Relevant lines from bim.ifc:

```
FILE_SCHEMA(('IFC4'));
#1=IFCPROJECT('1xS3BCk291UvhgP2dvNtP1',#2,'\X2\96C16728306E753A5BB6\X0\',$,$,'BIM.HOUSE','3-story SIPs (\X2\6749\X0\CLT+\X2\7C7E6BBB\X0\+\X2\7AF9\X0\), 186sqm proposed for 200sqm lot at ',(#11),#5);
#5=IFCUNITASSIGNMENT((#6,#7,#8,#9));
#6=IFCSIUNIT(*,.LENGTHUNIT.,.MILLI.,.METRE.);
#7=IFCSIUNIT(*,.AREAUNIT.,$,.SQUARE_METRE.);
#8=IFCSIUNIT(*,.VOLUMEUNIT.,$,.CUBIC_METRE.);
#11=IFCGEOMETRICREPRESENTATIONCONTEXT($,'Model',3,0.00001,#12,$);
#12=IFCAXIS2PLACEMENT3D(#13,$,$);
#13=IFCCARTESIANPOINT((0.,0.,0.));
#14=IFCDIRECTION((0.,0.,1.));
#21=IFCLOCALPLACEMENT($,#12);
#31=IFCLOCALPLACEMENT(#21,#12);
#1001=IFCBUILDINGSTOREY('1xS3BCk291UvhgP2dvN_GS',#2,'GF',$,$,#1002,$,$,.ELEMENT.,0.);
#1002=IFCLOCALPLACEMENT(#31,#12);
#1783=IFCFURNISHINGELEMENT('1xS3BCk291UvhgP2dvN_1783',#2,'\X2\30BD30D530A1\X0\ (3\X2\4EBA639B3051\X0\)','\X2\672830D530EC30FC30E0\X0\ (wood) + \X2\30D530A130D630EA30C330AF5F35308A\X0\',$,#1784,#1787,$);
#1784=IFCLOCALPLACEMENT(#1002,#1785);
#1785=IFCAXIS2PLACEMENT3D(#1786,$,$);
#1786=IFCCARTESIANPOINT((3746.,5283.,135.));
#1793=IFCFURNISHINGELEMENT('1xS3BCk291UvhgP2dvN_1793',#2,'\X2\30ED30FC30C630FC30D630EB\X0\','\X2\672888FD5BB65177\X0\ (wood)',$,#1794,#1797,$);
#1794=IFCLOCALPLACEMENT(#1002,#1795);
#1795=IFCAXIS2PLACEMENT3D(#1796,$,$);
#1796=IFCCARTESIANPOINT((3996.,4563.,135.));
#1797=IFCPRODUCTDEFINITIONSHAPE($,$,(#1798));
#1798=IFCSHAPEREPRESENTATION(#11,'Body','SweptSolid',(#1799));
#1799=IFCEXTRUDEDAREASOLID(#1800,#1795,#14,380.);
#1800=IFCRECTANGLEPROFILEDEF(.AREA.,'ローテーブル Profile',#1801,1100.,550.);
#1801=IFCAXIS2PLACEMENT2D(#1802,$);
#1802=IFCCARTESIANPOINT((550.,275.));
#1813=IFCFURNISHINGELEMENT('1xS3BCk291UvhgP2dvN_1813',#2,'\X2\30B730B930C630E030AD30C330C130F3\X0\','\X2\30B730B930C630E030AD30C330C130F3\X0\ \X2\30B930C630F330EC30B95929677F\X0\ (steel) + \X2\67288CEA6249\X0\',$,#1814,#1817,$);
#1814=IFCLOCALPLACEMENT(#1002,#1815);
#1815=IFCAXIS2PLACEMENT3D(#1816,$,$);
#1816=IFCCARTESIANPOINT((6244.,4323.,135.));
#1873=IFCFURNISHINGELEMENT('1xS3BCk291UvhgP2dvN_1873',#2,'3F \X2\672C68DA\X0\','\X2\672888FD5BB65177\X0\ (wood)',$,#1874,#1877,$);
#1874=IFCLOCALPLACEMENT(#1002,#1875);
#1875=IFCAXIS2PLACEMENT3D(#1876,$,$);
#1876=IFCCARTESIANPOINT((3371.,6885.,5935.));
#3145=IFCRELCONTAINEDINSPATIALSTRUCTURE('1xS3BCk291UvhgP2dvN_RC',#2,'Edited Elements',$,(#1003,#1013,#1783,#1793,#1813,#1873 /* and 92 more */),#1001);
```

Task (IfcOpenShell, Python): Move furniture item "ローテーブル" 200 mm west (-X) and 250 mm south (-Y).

```python
import ifcopenshell
import ifcopenshell.api.geometry
import ifcopenshell.util.placement
import ifcopenshell.util.unit

model = ifcopenshell.open("bim.ifc")
unit_scale = ifcopenshell.util.unit.calculate_unit_scale(model)

item = model.by_guid("1xS3BCk291UvhgP2dvN_1793")
matrix = ifcopenshell.util.placement.get_local_placement(item.ObjectPlacement)
matrix[0, 3] -= 0.2 / unit_scale
matrix[1, 3] -= 0.25 / unit_scale
ifcopenshell.api.geometry.edit_object_placement(model, product=item, matrix=matrix, is_si=False)

print(ifcopenshell.util.placement.get_local_placement(item.ObjectPlacement).round(3) + 0.0)

model.write("bim_updated.ifc")
```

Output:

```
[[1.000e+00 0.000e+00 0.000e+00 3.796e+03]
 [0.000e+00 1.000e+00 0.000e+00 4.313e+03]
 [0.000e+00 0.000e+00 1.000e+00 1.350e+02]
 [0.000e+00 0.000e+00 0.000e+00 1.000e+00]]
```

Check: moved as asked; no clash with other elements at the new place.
